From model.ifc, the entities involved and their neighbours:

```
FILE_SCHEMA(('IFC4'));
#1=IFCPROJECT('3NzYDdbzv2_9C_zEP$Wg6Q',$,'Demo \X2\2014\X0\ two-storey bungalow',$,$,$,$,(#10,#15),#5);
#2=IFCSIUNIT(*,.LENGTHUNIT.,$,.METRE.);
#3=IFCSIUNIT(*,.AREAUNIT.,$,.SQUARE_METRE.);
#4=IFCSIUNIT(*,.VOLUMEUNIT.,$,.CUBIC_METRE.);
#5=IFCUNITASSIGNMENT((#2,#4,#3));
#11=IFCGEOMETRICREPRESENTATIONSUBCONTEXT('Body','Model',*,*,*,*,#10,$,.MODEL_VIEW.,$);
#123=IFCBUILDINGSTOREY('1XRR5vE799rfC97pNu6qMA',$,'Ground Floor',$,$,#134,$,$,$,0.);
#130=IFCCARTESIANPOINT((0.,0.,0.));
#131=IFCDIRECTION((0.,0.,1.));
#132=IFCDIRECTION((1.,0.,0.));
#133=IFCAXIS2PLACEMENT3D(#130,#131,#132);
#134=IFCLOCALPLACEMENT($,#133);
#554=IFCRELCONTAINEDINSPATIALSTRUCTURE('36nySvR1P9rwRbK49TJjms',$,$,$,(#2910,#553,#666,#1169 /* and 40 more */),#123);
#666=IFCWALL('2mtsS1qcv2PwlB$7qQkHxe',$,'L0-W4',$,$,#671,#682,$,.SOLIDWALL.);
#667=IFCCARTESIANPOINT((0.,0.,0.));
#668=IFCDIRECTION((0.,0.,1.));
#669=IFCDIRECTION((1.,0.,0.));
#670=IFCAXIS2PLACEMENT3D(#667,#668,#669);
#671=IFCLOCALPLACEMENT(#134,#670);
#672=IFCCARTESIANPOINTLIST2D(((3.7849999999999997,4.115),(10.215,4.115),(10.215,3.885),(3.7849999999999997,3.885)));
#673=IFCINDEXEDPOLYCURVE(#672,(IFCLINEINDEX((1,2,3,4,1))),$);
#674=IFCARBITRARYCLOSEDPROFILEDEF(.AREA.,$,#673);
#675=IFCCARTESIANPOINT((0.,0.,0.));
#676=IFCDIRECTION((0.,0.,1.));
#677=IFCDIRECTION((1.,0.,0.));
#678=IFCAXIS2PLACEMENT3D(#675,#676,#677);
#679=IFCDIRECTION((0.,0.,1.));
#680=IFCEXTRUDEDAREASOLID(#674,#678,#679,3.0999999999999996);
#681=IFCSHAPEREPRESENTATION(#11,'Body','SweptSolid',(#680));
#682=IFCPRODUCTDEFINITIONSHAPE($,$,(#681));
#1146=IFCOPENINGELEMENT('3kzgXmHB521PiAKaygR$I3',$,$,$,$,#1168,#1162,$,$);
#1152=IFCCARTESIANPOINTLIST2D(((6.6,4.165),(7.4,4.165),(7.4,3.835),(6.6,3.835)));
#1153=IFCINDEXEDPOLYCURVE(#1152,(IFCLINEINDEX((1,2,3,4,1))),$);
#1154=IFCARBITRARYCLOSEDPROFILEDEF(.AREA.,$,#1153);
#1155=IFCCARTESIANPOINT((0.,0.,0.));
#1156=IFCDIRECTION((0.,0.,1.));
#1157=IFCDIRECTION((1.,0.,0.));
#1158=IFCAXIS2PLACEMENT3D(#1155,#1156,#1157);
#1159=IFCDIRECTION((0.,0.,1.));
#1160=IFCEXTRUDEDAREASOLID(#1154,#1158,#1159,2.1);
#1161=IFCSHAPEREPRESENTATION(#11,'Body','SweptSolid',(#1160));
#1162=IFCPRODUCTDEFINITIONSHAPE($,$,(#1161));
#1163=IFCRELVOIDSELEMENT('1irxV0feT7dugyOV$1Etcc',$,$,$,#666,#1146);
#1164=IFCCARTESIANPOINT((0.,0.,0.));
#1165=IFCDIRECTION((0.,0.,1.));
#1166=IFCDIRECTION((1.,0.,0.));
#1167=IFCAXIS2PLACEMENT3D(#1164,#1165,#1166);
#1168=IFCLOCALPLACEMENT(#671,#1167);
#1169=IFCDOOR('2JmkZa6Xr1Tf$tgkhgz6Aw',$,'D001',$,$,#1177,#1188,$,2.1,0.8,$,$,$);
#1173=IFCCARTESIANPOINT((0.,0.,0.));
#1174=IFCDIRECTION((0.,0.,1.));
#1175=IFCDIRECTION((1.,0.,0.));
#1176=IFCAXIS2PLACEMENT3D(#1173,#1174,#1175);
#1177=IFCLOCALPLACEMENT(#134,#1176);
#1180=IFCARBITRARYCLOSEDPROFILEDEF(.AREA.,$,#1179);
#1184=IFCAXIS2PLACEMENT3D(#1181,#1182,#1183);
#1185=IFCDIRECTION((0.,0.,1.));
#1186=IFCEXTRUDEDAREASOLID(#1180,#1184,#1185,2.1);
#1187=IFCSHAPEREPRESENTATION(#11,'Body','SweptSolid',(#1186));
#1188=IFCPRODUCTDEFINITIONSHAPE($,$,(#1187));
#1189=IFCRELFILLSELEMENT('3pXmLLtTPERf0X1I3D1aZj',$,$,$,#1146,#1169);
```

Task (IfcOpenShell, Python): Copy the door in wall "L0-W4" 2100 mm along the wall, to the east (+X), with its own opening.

```python
import ifcopenshell
import ifcopenshell.api.feature
import ifcopenshell.api.geometry
import ifcopenshell.api.root
import ifcopenshell.geom
import ifcopenshell.util.element
import ifcopenshell.util.placement
import ifcopenshell.util.shape
import ifcopenshell.util.unit

model = ifcopenshell.open("model.ifc")
unit_scale = ifcopenshell.util.unit.calculate_unit_scale(model)
settings = ifcopenshell.geom.settings()


def volume(element):
    """Net volume in cubic metres, openings subtracted."""
    shape = ifcopenshell.geom.create_shape(settings, element)
    return ifcopenshell.util.shape.get_volume(shape.geometry)


door = model.by_id(1169)
opening = door.FillsVoids[0].RelatingOpeningElement
wall = opening.VoidsElements[0].RelatingBuildingElement
before = volume(wall)
shift = ifcopenshell.util.placement.get_local_placement(wall.ObjectPlacement)[:3, 0] * 2.1 / unit_scale

# copy_class copies the void relationship, type, container and properties, but no geometry.
new_opening = ifcopenshell.api.root.copy_class(model, product=opening)
new_opening.Representation = ifcopenshell.util.element.copy_deep(
    model, opening.Representation, exclude=["IfcGeometricRepresentationContext", "IfcRepresentationMap"]
)
new_door = ifcopenshell.api.root.copy_class(model, product=door)
new_door.Representation = ifcopenshell.util.element.copy_deep(
    model, door.Representation, exclude=["IfcGeometricRepresentationContext", "IfcRepresentationMap"]
)
ifcopenshell.api.feature.add_filling(model, opening=new_opening, element=new_door)

for old, new in ((opening, new_opening), (door, new_door)):
    matrix = ifcopenshell.util.placement.get_local_placement(old.ObjectPlacement)
    matrix[:3, 3] += shift
    ifcopenshell.api.geometry.edit_object_placement(model, product=new, matrix=matrix, is_si=False)

after = volume(wall)

print(f"wall volume {before:.3f} -> {after:.3f} m3")

model.write("model_edited.ifc")
```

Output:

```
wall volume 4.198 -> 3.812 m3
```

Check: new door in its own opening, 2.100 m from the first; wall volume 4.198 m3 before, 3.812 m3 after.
